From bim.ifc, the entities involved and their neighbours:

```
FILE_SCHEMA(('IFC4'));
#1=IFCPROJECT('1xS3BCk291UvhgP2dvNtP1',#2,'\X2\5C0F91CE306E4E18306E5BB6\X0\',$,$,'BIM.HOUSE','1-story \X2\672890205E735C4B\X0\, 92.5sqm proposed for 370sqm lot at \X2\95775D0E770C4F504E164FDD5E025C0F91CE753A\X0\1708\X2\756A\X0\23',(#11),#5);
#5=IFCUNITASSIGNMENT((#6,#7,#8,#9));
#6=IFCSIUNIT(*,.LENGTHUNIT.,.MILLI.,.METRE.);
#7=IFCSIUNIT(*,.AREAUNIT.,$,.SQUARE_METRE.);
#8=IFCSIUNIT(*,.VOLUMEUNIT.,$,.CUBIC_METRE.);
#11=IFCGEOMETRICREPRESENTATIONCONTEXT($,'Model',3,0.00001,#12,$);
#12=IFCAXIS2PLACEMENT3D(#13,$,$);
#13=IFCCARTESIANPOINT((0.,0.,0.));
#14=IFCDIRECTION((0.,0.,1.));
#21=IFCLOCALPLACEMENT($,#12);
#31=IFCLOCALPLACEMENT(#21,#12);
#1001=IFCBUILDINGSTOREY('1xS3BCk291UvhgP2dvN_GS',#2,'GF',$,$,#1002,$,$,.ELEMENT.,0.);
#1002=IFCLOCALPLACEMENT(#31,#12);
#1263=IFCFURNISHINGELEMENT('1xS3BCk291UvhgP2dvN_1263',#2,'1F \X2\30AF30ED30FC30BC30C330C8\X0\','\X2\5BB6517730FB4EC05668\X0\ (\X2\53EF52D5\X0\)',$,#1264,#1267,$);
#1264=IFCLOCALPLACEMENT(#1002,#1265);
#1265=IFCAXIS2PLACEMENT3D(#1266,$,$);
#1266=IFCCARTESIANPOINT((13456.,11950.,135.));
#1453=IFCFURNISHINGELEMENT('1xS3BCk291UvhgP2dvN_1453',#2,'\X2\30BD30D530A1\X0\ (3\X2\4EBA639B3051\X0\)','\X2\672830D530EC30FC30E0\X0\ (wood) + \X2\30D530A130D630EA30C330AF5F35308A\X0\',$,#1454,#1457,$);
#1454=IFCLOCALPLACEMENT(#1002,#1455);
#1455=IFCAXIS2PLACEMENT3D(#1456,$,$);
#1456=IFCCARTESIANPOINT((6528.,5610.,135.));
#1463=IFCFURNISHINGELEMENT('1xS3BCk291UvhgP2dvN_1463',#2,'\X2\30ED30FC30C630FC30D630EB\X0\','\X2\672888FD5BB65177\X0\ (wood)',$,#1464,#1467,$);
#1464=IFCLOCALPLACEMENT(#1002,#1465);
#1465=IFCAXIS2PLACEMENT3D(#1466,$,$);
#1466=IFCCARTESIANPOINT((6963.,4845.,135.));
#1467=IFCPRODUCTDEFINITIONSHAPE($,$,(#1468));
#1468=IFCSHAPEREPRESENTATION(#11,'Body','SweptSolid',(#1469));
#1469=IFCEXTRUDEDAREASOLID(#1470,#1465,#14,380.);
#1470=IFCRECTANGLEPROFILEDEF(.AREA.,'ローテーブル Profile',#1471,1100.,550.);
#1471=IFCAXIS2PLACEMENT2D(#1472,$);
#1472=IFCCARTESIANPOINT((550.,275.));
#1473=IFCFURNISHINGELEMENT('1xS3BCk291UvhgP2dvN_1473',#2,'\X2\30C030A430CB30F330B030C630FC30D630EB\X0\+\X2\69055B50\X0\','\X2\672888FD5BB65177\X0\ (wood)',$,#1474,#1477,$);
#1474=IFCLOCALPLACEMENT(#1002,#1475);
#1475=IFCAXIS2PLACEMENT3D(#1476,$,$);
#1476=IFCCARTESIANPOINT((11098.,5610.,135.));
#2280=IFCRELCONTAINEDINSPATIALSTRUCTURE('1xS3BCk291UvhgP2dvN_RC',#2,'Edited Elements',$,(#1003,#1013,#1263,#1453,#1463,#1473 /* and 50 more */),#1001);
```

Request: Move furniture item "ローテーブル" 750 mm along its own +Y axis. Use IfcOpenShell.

```python
import ifcopenshell
import ifcopenshell.api.geometry
import ifcopenshell.util.placement
import ifcopenshell.util.unit

model = ifcopenshell.open("bim.ifc")
unit_scale = ifcopenshell.util.unit.calculate_unit_scale(model)

item = model.by_guid("1xS3BCk291UvhgP2dvN_1463")
matrix = ifcopenshell.util.placement.get_local_placement(item.ObjectPlacement)
matrix[:3, 3] += matrix[:3, 1] * 0.75 / unit_scale
ifcopenshell.api.geometry.edit_object_placement(model, product=item, matrix=matrix, is_si=False)

print(ifcopenshell.util.placement.get_local_placement(item.ObjectPlacement).round(3) + 0.0)

model.write("bim_edited.ifc")
```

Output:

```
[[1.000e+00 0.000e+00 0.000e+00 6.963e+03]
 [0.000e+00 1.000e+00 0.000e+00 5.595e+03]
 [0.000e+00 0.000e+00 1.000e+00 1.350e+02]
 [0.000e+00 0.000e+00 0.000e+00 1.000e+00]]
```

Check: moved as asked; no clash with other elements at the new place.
